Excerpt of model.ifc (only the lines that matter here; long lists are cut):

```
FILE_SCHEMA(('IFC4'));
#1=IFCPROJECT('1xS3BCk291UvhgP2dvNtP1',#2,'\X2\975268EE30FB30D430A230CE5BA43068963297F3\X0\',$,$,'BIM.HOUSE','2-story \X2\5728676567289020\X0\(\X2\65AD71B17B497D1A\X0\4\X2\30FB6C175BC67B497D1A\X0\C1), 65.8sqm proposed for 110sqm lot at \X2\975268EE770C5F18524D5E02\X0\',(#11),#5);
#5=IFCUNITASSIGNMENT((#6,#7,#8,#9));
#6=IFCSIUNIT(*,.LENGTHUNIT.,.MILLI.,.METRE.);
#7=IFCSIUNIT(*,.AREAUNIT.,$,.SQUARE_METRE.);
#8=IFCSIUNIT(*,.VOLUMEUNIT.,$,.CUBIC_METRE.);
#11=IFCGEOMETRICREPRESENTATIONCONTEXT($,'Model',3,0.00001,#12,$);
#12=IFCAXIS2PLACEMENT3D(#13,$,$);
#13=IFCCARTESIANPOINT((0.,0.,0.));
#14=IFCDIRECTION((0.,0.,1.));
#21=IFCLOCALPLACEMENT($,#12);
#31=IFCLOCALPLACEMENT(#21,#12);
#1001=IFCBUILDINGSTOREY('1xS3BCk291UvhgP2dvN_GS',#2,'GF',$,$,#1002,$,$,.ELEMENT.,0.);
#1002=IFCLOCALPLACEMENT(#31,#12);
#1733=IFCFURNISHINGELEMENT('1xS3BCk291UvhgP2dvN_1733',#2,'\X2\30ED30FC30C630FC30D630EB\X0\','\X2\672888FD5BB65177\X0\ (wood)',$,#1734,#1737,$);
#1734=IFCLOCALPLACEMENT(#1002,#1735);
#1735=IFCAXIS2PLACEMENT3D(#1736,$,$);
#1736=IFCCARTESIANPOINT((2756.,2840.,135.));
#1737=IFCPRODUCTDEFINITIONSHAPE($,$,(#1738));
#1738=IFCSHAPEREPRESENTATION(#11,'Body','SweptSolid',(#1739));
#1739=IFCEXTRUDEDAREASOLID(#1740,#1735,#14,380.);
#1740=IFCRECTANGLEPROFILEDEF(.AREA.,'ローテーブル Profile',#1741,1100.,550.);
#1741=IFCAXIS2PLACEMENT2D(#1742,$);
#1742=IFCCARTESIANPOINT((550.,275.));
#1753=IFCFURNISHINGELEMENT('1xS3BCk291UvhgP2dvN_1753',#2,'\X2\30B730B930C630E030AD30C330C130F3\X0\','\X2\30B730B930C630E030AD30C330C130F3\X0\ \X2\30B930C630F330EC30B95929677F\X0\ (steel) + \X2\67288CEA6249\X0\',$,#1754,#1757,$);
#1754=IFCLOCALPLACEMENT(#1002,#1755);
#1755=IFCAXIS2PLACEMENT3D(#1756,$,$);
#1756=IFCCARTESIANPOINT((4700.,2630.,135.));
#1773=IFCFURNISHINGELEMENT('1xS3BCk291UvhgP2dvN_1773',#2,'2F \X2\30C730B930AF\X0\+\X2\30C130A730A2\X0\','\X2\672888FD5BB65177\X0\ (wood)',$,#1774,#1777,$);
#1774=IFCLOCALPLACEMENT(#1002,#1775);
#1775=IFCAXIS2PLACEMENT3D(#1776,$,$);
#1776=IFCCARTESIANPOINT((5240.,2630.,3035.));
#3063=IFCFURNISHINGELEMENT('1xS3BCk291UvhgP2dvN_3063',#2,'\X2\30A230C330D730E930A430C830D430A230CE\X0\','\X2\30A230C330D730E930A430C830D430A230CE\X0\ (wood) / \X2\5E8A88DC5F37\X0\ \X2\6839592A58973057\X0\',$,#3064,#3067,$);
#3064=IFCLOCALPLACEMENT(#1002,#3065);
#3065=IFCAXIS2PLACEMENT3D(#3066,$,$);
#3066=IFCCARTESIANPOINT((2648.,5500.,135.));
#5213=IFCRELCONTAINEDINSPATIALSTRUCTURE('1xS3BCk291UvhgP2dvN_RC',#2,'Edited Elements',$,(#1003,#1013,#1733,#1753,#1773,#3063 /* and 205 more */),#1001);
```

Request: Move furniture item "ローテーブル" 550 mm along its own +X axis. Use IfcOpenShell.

```python
import ifcopenshell
import ifcopenshell.api.geometry
import ifcopenshell.util.placement

model = ifcopenshell.open("model.ifc")

item = model.by_guid("1xS3BCk291UvhgP2dvN_1733")
matrix = ifcopenshell.util.placement.get_local_placement(item.ObjectPlacement)
matrix[:3, 3] += matrix[:3, 0] * 550.0
ifcopenshell.api.geometry.edit_object_placement(model, product=item, matrix=matrix, is_si=False)

print(ifcopenshell.util.placement.get_local_placement(item.ObjectPlacement).round(3) + 0.0)

model.write("model_v2.ifc")
```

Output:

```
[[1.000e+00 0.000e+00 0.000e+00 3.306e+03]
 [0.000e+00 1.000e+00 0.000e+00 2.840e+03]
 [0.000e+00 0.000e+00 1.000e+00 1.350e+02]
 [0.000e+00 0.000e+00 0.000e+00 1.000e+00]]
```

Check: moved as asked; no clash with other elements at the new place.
